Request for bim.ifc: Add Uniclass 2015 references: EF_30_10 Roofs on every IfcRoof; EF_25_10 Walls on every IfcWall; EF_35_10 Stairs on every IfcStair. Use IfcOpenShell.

First a look at what the model holds.

```python
import ifcopenshell

model = ifcopenshell.open("bim.ifc")
print(model.schema)
print("classifications:", [c.Name for c in model.by_type("IfcClassification")])
for ifc_class in ("IfcDoor", "IfcRoof", "IfcStair", "IfcWall", "IfcWindow"):
    print(ifc_class, len(model.by_type(ifc_class)))
```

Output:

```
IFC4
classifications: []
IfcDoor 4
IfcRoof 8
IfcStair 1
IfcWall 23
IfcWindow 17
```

```python
import ifcopenshell
import ifcopenshell.api.classification

model = ifcopenshell.open("bim.ifc")

system = ifcopenshell.api.classification.add_classification(model, classification="Uniclass 2015")

codes = {
    "IfcRoof": ("EF_30_10", "Roofs"),
    "IfcWall": ("EF_25_10", "Walls"),
    "IfcStair": ("EF_35_10", "Stairs"),
}
for ifc_class, (code, name) in codes.items():
    products = model.by_type(ifc_class)
    ifcopenshell.api.classification.add_reference(
        model, products=products, classification=system, identification=code, name=name
    )
    print(code, len(products))

model.write("bim_edited.ifc")
```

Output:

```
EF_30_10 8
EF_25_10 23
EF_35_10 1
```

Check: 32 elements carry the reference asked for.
